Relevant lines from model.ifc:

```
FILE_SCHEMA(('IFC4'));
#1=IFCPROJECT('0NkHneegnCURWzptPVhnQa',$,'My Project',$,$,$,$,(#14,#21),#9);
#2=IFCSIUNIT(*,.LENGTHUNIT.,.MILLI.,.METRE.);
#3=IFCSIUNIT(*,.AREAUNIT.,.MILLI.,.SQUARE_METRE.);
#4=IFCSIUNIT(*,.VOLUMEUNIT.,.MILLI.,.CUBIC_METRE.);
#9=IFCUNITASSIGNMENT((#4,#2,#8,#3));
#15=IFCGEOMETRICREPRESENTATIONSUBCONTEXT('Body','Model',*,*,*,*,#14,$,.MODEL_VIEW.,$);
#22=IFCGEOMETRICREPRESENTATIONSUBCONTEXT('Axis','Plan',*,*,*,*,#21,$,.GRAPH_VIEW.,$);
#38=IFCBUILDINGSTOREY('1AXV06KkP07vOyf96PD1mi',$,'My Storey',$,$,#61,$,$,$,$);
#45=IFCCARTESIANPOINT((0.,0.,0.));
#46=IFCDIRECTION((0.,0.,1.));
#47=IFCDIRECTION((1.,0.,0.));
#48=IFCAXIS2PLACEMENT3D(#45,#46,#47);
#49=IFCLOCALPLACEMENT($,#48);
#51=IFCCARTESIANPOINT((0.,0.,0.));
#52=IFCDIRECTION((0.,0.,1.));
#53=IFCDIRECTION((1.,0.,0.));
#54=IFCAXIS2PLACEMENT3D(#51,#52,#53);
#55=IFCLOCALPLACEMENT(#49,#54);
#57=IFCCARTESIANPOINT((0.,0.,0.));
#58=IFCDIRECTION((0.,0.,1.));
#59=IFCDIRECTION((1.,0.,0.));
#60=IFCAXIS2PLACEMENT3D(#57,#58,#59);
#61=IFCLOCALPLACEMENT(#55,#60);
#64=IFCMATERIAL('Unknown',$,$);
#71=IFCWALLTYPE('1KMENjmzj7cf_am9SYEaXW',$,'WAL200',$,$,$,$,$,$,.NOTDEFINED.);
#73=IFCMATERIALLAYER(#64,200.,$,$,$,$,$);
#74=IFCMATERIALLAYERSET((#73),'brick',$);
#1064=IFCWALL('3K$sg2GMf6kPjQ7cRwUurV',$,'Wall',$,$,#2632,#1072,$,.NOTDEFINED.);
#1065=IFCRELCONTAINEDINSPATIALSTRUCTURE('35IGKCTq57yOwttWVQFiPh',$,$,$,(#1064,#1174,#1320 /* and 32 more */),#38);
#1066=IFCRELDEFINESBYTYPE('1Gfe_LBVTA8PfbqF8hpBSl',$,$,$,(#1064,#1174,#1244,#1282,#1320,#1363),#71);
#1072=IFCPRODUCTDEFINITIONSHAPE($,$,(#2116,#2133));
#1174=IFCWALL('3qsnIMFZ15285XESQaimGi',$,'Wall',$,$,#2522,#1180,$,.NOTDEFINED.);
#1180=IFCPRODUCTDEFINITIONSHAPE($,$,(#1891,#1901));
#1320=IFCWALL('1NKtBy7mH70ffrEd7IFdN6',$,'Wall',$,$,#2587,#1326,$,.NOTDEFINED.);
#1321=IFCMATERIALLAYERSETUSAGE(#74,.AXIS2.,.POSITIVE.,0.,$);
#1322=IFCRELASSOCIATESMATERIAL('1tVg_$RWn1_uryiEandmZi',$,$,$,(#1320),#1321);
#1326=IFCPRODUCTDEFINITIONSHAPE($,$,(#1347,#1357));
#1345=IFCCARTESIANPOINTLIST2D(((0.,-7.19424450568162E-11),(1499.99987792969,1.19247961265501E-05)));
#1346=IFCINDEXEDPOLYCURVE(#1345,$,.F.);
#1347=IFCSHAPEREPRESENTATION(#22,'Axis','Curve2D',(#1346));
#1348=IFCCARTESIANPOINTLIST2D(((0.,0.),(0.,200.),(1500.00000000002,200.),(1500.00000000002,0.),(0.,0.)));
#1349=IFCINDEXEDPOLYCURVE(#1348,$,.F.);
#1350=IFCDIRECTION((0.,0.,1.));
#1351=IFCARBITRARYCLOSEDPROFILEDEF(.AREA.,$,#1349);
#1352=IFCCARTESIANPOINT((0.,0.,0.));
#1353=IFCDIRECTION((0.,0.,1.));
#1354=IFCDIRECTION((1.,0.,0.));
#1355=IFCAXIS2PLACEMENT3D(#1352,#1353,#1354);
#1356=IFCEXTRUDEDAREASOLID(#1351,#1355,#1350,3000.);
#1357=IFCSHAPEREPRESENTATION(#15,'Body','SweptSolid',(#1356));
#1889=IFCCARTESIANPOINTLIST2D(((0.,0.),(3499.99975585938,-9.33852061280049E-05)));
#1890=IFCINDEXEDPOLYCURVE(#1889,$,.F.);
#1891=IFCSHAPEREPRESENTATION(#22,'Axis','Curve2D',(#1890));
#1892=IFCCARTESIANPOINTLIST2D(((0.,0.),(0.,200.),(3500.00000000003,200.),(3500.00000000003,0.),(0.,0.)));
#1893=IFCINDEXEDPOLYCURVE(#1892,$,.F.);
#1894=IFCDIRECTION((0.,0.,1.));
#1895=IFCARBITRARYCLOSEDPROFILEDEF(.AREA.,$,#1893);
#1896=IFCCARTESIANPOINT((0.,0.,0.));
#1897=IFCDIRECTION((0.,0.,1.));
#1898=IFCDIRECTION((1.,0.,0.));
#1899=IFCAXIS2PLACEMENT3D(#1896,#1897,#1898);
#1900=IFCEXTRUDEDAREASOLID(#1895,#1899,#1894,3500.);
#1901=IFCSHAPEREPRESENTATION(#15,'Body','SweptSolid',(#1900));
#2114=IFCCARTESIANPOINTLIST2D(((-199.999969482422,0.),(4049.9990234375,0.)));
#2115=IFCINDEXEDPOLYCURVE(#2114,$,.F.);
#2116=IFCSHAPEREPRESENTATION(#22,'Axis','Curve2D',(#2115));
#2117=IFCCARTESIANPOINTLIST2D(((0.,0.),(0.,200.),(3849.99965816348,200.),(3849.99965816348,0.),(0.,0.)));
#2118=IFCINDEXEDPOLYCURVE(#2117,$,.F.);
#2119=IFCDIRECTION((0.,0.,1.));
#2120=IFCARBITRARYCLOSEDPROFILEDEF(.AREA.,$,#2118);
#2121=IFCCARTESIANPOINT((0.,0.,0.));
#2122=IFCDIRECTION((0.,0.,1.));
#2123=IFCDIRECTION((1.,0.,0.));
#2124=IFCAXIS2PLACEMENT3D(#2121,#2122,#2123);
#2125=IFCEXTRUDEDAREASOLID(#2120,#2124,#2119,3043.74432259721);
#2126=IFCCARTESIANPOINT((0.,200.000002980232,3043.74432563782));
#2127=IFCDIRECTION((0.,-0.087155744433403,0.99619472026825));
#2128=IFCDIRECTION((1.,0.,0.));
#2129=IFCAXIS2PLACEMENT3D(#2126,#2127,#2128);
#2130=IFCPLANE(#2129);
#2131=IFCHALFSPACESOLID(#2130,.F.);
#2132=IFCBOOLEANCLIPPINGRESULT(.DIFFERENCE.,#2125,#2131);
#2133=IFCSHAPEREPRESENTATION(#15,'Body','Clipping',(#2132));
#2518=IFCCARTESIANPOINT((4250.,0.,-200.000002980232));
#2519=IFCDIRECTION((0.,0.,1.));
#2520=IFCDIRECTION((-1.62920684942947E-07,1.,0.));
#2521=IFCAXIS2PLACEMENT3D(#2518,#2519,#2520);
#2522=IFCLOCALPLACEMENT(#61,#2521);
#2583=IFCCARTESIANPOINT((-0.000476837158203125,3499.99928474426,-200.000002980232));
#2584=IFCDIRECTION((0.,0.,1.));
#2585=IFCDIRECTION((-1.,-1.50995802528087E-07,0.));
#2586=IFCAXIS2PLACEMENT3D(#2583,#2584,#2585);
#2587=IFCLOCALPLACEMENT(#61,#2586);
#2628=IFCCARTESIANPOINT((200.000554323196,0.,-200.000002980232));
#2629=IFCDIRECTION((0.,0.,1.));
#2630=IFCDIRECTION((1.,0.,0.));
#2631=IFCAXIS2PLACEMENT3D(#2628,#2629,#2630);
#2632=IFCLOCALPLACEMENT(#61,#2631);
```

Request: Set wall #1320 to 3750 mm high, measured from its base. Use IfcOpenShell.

```python
import ifcopenshell
import ifcopenshell.geom
import ifcopenshell.util.representation
import ifcopenshell.util.shape
import ifcopenshell.util.unit

model = ifcopenshell.open("model.ifc")
unit_scale = ifcopenshell.util.unit.calculate_unit_scale(model)
settings = ifcopenshell.geom.settings()


def volume(element):
    """Net volume in cubic metres, openings subtracted."""
    shape = ifcopenshell.geom.create_shape(settings, element)
    return ifcopenshell.util.shape.get_volume(shape.geometry)


wall = model.by_guid("1NKtBy7mH70ffrEd7IFdN6")
before = volume(wall)

body = ifcopenshell.util.representation.get_representation(wall, "Model", "Body")
solid = body.Items[0]
old_height = solid.Depth
solid.Depth = 3.75 / unit_scale
after = volume(wall)

print(f"height {old_height:g} -> {solid.Depth:g}, volume {before:.3f} -> {after:.3f} m3")

model.write("model-out.ifc")
```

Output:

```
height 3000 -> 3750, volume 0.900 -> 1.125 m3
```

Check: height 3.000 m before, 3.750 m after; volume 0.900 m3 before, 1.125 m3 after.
